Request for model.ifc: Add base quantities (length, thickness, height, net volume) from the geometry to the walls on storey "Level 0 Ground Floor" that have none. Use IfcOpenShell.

First a look at what the model holds.

```python
import ifcopenshell
import ifcopenshell.util.element
import ifcopenshell.util.unit

model = ifcopenshell.open("model.ifc")
print(model.schema)
for unit_type in ("LENGTHUNIT", "AREAUNIT", "VOLUMEUNIT"):
    print(unit_type, ifcopenshell.util.unit.calculate_unit_scale(model, unit_type))
storey = next(s for s in model.by_type("IfcBuildingStorey") if s.Name == "Level 0 Ground Floor")
walls = [e for e in ifcopenshell.util.element.get_decomposition(storey) if e.is_a("IfcWall")]
for e in sorted(walls, key=lambda e: e.id()):
    print(e.id(), e.is_a(), e.Name, list(ifcopenshell.util.element.get_psets(e, qtos_only=True)), sep=" | ")
```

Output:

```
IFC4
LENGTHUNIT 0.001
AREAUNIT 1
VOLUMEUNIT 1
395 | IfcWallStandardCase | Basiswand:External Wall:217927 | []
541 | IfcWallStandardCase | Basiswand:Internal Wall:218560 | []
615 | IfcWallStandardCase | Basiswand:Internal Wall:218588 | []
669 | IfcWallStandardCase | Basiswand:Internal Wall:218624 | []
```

```python
import ifcopenshell
import ifcopenshell.api.pset
import ifcopenshell.geom
import ifcopenshell.util.element
import ifcopenshell.util.shape
import ifcopenshell.util.unit

model = ifcopenshell.open("model.ifc")
unit_scale = ifcopenshell.util.unit.calculate_unit_scale(model)
volume_scale = ifcopenshell.util.unit.calculate_unit_scale(model, "VOLUMEUNIT")
settings = ifcopenshell.geom.settings()

storey = next(s for s in model.by_type("IfcBuildingStorey") if s.Name == "Level 0 Ground Floor")
walls = [e for e in ifcopenshell.util.element.get_decomposition(storey) if e.is_a("IfcWall")]

for e in sorted(walls, key=lambda e: e.id()):
    if ifcopenshell.util.element.get_psets(e, qtos_only=True, should_inherit=False):
        continue
    # Geometry comes back in metres, in the element's own axes.
    shape = ifcopenshell.geom.create_shape(settings, e)
    values = {
        "Length": ifcopenshell.util.shape.get_x(shape.geometry) / unit_scale,
        "Width": ifcopenshell.util.shape.get_y(shape.geometry) / unit_scale,
        "Height": ifcopenshell.util.shape.get_z(shape.geometry) / unit_scale,
        "NetVolume": ifcopenshell.util.shape.get_volume(shape.geometry) / volume_scale,
    }
    qto = ifcopenshell.api.pset.add_qto(model, product=e, name="Qto_WallBaseQuantities")
    ifcopenshell.api.pset.edit_qto(model, qto=qto, properties=values)
    print(e.id(), {k: round(v, 3) for k, v in values.items()})

model.write("model_edited.ifc")
```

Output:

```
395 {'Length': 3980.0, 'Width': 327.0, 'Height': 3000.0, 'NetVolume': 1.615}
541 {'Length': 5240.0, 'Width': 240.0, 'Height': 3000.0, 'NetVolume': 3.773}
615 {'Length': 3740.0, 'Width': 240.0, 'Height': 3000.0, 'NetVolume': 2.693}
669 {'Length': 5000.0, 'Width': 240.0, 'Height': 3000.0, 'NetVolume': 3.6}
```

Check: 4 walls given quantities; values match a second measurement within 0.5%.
